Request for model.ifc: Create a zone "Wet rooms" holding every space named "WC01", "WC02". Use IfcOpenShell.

First a look at what the model holds.

```python
import ifcopenshell

model = ifcopenshell.open("model.ifc")
print(model.schema)
seen = {}
for space in model.by_type("IfcSpace"):
    seen[space.LongName] = seen.get(space.LongName, 0) + 1
for name, count in sorted(seen.items(), key=str):
    print(count, "x", name)
print("zones:", [z.Name for z in model.by_type("IfcZone")][:20])
```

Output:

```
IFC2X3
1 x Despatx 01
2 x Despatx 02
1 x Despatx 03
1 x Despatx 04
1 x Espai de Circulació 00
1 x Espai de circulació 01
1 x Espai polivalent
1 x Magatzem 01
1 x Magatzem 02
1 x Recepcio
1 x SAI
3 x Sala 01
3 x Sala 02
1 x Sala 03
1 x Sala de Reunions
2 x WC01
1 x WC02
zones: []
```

```python
import ifcopenshell
import ifcopenshell.api.group
import ifcopenshell.api.root

model = ifcopenshell.open("model.ifc")

names = {"WC01", "WC02"}
spaces = [s for s in model.by_type("IfcSpace") if s.LongName in names]

zone = ifcopenshell.api.root.create_entity(model, ifc_class="IfcZone", name="Wet rooms")
ifcopenshell.api.group.assign_group(model, products=spaces, group=zone)
print(len(spaces), "spaces in", zone.Name)

model.write("model_rev.ifc")
```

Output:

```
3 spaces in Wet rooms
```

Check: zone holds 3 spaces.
